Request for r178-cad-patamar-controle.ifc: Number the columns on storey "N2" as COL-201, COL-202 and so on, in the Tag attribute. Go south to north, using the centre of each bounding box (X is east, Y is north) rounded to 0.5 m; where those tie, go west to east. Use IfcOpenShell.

First a look at what the model holds.

```python
import ifcopenshell
import ifcopenshell.util.element
import ifcopenshell.util.placement

model = ifcopenshell.open("r178-cad-patamar-controle.ifc")
print(model.schema)
storey = next(s for s in model.by_type("IfcBuildingStorey") if s.Name == "N2")
columns = [e for e in ifcopenshell.util.element.get_decomposition(storey) if e.is_a("IfcColumn")]
for e in sorted(columns, key=lambda e: e.id()):
    origin = ifcopenshell.util.placement.get_local_placement(e.ObjectPlacement)[:3, 3]
    print(e.id(), e.Tag, e.Name, origin.round(2) + 0.0, sep=" | ")
```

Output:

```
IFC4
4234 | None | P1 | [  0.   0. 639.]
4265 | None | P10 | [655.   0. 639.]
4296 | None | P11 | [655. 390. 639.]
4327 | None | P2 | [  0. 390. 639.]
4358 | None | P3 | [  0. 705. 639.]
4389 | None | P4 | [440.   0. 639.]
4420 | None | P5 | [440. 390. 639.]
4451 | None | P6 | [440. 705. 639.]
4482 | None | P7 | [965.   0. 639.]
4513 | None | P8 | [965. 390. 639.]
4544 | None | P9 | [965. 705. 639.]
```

```python
import ifcopenshell
import ifcopenshell.geom
import ifcopenshell.util.element
import ifcopenshell.util.shape

model = ifcopenshell.open("r178-cad-patamar-controle.ifc")
settings = ifcopenshell.geom.settings()
settings.set("use-world-coords", True)


def centre(element):
    shape = ifcopenshell.geom.create_shape(settings, element)
    return ifcopenshell.util.shape.get_bbox_centroid(shape.geometry)


storey = next(s for s in model.by_type("IfcBuildingStorey") if s.Name == "N2")
columns = [e for e in ifcopenshell.util.element.get_decomposition(storey) if e.is_a("IfcColumn")]

# Insertion points can sit at a corner or the storey origin, so sort by the geometry (in metres).
centres = {e: centre(e) for e in columns}
columns.sort(key=lambda e: (round(centres[e][1] / 0.5), centres[e][0]))

for i, e in enumerate(columns, start=1):
    number = f"COL-2{i:02d}"
    e.Tag = number
    print(e.id(), number)

model.write("r178-cad-patamar-controle_v2.ifc")
```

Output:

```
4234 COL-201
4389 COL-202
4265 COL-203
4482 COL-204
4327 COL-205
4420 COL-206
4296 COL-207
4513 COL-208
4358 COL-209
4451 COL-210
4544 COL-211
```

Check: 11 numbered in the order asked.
